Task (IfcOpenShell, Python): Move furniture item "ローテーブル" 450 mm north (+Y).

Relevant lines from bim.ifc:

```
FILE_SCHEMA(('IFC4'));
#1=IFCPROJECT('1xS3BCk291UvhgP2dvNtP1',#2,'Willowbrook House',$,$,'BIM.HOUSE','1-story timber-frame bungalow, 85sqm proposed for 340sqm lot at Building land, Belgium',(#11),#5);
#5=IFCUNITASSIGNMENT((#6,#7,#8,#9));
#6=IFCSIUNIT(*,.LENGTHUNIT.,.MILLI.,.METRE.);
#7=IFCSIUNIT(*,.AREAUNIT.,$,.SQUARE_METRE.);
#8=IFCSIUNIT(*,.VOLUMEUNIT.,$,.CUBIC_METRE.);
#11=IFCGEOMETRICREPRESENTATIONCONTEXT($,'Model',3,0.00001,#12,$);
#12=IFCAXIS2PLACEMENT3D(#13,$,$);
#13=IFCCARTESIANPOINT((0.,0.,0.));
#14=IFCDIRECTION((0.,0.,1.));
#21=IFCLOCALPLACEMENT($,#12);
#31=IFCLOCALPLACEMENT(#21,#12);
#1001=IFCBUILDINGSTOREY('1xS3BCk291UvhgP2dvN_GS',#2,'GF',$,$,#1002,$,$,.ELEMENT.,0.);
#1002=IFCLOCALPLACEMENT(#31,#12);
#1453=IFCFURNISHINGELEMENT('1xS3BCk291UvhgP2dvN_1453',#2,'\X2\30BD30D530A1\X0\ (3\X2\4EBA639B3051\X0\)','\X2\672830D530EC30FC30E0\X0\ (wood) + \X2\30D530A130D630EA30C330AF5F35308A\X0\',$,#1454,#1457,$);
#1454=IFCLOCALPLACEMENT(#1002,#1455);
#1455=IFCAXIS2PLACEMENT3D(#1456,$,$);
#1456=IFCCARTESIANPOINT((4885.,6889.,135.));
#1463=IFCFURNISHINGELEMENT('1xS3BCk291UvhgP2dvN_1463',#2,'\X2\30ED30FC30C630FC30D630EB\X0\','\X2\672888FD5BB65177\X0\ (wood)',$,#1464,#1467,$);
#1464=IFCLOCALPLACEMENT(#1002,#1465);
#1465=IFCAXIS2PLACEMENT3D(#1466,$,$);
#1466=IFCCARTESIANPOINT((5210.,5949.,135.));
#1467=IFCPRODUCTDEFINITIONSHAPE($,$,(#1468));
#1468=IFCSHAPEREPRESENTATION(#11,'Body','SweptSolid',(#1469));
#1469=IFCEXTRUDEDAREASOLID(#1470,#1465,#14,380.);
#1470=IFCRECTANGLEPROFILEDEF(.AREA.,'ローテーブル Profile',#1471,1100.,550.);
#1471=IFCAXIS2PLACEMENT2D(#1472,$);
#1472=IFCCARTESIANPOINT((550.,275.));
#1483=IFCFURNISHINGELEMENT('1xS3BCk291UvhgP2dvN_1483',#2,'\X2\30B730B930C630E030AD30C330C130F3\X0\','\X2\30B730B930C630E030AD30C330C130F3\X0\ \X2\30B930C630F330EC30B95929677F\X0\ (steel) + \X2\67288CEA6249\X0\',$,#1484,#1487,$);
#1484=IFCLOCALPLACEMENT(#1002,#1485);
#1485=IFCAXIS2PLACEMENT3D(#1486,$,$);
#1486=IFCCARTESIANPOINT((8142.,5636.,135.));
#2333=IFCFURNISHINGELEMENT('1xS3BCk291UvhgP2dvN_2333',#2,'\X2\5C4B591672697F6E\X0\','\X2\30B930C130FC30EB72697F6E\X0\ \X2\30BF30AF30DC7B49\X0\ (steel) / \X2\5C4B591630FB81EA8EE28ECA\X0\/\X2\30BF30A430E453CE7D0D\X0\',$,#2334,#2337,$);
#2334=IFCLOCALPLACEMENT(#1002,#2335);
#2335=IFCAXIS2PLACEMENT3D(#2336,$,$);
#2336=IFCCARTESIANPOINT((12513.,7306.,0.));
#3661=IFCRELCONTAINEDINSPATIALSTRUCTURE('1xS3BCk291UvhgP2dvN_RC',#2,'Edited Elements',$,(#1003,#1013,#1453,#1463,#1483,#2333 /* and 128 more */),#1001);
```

```python
import ifcopenshell
import ifcopenshell.api.geometry
import ifcopenshell.util.placement
import ifcopenshell.util.unit

model = ifcopenshell.open("bim.ifc")
unit_scale = ifcopenshell.util.unit.calculate_unit_scale(model)

item = model.by_guid("1xS3BCk291UvhgP2dvN_1463")
matrix = ifcopenshell.util.placement.get_local_placement(item.ObjectPlacement)
matrix[1, 3] += 0.45 / unit_scale
ifcopenshell.api.geometry.edit_object_placement(model, product=item, matrix=matrix, is_si=False)

print(ifcopenshell.util.placement.get_local_placement(item.ObjectPlacement).round(3) + 0.0)

model.write("bim_rev.ifc")
```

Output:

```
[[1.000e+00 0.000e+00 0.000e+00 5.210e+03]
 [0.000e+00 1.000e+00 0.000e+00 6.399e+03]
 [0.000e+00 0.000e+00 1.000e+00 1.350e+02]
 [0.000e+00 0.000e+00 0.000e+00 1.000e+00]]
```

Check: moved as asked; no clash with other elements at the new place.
